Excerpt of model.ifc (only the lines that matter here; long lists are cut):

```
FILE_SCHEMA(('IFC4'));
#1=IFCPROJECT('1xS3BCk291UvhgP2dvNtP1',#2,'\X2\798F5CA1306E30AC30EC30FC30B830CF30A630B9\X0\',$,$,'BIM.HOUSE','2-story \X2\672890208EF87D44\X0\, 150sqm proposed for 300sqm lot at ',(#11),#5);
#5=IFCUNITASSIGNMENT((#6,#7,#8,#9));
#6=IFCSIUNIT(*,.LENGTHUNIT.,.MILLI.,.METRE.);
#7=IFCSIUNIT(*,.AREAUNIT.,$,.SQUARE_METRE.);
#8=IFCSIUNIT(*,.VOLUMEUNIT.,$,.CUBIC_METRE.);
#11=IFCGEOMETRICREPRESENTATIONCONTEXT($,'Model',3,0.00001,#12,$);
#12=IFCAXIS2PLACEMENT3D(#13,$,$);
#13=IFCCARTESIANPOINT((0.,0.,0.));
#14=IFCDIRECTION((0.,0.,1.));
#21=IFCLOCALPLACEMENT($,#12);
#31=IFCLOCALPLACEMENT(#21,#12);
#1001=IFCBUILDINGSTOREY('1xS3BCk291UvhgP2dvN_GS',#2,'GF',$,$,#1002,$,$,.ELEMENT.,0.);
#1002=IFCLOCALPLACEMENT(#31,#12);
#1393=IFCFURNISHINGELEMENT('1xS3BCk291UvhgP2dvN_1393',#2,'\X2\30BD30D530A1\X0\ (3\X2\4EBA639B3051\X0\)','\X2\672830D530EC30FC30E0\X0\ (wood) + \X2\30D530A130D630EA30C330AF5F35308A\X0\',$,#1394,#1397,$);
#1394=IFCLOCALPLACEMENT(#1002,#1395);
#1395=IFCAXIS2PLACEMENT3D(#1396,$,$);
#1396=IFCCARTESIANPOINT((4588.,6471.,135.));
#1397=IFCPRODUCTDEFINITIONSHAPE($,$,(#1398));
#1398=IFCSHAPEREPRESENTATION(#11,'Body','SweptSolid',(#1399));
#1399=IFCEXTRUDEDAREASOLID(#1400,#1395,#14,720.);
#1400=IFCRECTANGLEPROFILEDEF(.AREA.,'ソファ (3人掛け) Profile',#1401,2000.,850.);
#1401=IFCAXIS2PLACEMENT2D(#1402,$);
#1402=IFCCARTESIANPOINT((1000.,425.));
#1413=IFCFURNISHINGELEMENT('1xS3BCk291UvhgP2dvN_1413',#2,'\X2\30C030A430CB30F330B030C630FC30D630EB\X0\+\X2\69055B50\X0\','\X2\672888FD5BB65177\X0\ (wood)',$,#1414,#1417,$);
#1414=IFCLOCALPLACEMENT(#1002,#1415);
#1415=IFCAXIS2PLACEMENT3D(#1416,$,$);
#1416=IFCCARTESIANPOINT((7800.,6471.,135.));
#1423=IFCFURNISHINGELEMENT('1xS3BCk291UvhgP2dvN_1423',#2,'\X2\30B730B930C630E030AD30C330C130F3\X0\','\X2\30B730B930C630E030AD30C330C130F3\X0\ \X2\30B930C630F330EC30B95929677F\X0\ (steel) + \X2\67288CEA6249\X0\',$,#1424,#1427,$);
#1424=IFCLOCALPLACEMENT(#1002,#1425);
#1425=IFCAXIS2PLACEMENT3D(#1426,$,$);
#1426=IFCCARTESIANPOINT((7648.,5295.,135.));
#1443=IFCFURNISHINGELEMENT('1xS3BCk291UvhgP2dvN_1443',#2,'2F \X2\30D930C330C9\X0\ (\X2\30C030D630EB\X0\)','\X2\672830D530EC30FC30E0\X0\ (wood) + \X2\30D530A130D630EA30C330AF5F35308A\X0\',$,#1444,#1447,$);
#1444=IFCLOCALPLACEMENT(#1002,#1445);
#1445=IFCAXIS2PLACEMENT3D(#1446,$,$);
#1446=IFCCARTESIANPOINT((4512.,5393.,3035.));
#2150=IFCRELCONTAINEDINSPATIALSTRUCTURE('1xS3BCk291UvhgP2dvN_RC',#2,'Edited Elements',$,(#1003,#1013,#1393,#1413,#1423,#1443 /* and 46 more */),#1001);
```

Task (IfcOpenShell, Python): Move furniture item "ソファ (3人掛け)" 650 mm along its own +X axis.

```python
import ifcopenshell
import ifcopenshell.api.geometry
import ifcopenshell.util.placement

model = ifcopenshell.open("model.ifc")

item = model.by_id(1393)
matrix = ifcopenshell.util.placement.get_local_placement(item.ObjectPlacement)
matrix[:3, 3] += matrix[:3, 0] * 650.0
ifcopenshell.api.geometry.edit_object_placement(model, product=item, matrix=matrix, is_si=False)

print(ifcopenshell.util.placement.get_local_placement(item.ObjectPlacement).round(3) + 0.0)

model.write("model_edited.ifc")
```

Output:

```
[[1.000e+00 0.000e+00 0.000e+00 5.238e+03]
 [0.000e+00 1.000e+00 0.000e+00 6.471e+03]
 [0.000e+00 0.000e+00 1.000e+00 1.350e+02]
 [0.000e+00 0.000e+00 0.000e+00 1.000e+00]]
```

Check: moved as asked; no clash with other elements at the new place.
